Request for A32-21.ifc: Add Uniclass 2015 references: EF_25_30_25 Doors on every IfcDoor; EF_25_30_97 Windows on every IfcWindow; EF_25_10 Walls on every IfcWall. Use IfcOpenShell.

First a look at what the model holds.

```python
import ifcopenshell

model = ifcopenshell.open("A32-21.ifc")
print(model.schema)
print("classifications:", [c.Name for c in model.by_type("IfcClassification")])
for ifc_class in ("IfcDoor", "IfcRoof", "IfcStair", "IfcWall", "IfcWindow"):
    print(ifc_class, len(model.by_type(ifc_class)))
```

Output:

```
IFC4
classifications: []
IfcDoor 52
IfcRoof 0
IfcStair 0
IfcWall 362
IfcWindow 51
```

```python
import ifcopenshell
import ifcopenshell.api.classification

model = ifcopenshell.open("A32-21.ifc")

system = ifcopenshell.api.classification.add_classification(model, classification="Uniclass 2015")

codes = {
    "IfcDoor": ("EF_25_30_25", "Doors"),
    "IfcWindow": ("EF_25_30_97", "Windows"),
    "IfcWall": ("EF_25_10", "Walls"),
}
for ifc_class, (code, name) in codes.items():
    products = model.by_type(ifc_class)
    ifcopenshell.api.classification.add_reference(
        model, products=products, classification=system, identification=code, name=name
    )
    print(code, len(products))

model.write("A32-21_edited.ifc")
```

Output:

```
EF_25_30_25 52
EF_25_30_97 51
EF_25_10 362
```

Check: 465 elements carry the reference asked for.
